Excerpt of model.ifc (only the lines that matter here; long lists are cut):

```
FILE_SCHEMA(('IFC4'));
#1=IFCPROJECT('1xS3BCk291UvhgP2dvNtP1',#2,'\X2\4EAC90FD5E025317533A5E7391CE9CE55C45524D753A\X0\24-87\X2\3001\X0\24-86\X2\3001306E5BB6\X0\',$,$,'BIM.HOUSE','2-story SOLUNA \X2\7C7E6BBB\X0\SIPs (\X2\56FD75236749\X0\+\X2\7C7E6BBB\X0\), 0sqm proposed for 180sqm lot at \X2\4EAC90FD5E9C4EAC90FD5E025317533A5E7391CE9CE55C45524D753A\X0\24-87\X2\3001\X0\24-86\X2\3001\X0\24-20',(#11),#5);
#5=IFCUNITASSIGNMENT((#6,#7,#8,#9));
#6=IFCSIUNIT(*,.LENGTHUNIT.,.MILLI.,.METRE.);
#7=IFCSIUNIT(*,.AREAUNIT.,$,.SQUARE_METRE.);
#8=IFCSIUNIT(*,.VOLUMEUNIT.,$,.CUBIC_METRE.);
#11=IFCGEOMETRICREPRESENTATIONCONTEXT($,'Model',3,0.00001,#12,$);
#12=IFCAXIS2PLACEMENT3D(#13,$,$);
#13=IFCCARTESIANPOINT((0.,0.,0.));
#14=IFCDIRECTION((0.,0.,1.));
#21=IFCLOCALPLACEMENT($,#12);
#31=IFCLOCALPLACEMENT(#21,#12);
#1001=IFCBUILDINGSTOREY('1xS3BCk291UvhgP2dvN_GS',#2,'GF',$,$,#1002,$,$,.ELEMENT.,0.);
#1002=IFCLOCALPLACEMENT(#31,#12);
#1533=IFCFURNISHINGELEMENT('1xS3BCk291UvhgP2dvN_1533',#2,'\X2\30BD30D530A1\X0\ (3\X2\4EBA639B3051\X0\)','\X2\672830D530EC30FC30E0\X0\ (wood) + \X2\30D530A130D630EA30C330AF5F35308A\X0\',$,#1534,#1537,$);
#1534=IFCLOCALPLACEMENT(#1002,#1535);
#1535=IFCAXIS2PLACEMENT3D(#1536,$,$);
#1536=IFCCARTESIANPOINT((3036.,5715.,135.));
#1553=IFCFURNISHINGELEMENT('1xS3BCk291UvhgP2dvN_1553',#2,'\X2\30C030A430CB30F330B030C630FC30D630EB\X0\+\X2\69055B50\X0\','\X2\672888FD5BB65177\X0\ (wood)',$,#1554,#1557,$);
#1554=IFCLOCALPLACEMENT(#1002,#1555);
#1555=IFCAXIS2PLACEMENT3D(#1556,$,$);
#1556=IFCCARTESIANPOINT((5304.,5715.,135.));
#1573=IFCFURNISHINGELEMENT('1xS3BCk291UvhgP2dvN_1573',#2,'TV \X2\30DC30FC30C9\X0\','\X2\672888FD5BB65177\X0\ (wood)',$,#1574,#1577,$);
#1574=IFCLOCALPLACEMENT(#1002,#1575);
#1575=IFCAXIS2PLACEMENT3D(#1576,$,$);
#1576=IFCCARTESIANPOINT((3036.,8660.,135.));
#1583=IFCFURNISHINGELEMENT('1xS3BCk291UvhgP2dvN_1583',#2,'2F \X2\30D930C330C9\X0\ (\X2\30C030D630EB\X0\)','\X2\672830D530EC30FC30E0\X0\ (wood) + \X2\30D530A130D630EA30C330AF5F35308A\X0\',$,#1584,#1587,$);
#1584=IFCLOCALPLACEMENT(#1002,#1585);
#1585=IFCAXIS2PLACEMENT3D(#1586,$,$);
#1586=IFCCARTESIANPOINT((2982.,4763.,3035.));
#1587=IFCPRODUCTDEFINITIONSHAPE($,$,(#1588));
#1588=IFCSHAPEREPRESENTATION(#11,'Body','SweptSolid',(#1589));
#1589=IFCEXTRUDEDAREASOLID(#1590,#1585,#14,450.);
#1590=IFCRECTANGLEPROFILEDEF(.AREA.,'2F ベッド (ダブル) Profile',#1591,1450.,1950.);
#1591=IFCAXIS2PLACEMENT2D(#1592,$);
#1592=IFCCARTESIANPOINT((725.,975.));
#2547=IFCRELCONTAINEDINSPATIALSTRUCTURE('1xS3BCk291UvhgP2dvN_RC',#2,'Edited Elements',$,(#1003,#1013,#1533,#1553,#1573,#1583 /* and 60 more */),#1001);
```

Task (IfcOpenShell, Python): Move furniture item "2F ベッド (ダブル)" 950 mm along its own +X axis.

```python
import ifcopenshell
import ifcopenshell.api.geometry
import ifcopenshell.util.placement
import ifcopenshell.util.unit

model = ifcopenshell.open("model.ifc")
unit_scale = ifcopenshell.util.unit.calculate_unit_scale(model)

item = model.by_guid("1xS3BCk291UvhgP2dvN_1583")
matrix = ifcopenshell.util.placement.get_local_placement(item.ObjectPlacement)
matrix[:3, 3] += matrix[:3, 0] * 0.95 / unit_scale
ifcopenshell.api.geometry.edit_object_placement(model, product=item, matrix=matrix, is_si=False)

print(ifcopenshell.util.placement.get_local_placement(item.ObjectPlacement).round(3) + 0.0)

model.write("model-out.ifc")
```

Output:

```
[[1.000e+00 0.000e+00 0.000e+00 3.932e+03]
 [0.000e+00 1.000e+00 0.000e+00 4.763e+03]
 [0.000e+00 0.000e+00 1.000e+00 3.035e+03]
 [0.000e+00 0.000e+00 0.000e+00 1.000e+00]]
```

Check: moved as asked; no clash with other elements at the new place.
